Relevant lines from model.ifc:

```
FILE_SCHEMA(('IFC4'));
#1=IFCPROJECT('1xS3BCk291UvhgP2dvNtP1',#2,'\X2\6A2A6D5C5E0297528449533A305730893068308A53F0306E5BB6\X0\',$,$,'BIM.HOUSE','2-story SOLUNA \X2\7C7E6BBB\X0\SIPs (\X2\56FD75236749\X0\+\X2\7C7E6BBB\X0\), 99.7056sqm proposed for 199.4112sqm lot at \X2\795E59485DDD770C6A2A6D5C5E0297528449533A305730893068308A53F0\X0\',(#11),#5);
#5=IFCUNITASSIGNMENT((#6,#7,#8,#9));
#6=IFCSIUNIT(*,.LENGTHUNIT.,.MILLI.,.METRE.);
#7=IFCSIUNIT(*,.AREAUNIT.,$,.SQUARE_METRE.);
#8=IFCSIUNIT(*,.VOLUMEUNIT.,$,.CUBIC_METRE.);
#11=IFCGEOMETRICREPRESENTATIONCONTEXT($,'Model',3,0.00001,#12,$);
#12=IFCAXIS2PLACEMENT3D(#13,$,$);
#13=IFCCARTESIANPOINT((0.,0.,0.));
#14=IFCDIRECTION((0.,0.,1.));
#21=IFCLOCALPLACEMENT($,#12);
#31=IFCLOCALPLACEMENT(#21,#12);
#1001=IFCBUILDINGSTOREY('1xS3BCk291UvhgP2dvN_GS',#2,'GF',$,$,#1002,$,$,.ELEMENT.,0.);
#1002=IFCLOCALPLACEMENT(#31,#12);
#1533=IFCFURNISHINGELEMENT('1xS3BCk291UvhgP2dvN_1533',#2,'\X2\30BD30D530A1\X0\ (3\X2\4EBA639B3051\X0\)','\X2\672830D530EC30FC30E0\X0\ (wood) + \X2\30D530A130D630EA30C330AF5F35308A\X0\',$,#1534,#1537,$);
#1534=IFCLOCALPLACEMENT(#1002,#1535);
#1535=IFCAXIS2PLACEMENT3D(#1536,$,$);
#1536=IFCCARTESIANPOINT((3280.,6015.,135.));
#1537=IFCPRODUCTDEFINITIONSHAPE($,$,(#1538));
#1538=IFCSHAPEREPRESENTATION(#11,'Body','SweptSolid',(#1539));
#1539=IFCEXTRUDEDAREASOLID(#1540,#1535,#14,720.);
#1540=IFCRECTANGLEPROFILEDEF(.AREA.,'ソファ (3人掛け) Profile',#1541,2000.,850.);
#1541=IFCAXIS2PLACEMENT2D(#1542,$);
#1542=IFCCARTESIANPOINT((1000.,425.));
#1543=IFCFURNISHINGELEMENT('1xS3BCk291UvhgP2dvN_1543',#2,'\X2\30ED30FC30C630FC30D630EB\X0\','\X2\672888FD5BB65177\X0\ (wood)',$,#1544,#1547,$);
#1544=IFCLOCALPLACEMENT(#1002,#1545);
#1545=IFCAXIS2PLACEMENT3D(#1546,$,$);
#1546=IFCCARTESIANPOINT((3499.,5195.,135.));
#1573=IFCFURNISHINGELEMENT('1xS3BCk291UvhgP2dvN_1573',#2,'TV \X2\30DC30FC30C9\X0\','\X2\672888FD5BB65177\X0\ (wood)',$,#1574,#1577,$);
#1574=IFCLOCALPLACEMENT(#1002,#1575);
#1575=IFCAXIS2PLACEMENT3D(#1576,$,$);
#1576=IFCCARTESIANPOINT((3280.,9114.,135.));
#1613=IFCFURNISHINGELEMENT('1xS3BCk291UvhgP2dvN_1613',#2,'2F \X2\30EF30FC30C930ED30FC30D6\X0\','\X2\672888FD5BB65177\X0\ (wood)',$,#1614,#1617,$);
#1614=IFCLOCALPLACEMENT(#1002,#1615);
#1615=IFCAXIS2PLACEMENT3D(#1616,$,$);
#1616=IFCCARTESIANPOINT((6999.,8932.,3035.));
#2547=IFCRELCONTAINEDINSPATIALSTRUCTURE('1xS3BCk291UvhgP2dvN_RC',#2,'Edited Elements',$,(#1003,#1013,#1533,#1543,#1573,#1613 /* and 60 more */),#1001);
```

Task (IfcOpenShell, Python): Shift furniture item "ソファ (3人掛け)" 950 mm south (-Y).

```python
import ifcopenshell
import ifcopenshell.api.geometry
import ifcopenshell.util.placement
import ifcopenshell.util.unit

model = ifcopenshell.open("model.ifc")
unit_scale = ifcopenshell.util.unit.calculate_unit_scale(model)

item = model.by_guid("1xS3BCk291UvhgP2dvN_1533")
matrix = ifcopenshell.util.placement.get_local_placement(item.ObjectPlacement)
matrix[1, 3] -= 0.95 / unit_scale
ifcopenshell.api.geometry.edit_object_placement(model, product=item, matrix=matrix, is_si=False)

print(ifcopenshell.util.placement.get_local_placement(item.ObjectPlacement).round(3) + 0.0)

model.write("model_edited.ifc")
```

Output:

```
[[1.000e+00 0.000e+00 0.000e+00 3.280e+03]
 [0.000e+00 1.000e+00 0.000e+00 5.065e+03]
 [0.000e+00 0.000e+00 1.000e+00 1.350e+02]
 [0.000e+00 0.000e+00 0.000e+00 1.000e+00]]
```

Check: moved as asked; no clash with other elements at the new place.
